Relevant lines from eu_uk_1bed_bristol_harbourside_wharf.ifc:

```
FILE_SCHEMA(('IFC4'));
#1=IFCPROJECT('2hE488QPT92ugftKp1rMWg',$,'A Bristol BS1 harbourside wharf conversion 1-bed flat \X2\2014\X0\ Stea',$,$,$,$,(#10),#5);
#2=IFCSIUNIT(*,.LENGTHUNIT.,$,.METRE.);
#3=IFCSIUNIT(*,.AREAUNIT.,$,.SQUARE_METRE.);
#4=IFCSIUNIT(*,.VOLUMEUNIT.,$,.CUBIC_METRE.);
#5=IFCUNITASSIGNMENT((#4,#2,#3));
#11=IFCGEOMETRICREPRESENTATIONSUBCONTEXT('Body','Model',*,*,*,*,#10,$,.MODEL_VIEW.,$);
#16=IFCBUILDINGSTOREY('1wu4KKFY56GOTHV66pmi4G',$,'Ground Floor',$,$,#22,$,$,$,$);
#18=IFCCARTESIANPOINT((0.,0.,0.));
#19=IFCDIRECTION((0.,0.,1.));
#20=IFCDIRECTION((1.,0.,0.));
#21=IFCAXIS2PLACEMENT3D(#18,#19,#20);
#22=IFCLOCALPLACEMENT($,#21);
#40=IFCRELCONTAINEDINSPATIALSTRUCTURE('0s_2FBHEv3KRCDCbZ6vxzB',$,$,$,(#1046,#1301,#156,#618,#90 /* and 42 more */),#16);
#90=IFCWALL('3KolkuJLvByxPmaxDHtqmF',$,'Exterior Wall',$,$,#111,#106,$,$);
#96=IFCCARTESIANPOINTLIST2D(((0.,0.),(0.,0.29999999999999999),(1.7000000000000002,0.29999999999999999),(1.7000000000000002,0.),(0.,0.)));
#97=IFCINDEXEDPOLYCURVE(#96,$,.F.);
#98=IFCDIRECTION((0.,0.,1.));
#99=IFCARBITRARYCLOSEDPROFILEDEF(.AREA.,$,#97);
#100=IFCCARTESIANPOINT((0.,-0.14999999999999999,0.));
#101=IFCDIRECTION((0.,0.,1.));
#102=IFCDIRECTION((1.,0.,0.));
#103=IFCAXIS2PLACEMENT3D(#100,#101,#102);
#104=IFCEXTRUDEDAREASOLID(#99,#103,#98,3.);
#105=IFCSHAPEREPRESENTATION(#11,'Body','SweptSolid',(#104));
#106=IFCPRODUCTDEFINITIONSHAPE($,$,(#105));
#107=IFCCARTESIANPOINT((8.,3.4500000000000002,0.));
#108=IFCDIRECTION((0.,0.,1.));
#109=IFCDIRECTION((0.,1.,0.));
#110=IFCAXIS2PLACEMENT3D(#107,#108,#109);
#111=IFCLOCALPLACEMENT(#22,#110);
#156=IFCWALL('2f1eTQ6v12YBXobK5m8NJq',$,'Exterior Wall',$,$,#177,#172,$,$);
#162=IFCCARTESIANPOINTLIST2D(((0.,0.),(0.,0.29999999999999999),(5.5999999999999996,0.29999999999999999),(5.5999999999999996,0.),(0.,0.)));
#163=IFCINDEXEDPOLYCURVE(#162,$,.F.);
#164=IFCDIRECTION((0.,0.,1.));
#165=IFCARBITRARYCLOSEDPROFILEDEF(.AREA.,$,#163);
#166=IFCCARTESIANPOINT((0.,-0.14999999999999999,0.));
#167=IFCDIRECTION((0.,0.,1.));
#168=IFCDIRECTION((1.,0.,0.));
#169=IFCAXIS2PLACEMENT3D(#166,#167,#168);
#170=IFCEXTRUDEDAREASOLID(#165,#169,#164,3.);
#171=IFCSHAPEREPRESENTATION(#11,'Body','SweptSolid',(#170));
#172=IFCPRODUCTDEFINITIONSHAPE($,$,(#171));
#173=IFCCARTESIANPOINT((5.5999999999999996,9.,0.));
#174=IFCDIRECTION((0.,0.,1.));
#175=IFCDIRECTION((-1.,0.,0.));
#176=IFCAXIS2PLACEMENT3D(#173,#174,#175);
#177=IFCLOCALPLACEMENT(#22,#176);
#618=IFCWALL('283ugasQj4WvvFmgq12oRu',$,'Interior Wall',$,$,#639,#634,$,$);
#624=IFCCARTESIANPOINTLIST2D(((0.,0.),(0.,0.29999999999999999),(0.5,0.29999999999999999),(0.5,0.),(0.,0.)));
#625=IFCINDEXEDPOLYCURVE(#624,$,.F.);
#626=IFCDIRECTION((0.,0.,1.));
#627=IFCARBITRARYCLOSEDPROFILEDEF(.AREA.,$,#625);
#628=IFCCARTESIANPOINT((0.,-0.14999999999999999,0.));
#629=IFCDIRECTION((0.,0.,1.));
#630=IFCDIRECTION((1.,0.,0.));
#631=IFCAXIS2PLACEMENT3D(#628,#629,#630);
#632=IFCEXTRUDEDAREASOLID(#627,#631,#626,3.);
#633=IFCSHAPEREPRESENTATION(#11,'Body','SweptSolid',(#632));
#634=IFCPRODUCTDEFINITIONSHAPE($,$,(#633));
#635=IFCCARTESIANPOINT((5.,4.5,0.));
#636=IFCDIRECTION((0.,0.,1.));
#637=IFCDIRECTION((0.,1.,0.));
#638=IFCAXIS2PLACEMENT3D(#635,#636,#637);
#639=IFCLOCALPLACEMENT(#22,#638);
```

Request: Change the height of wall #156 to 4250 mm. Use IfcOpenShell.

```python
import ifcopenshell
import ifcopenshell.geom
import ifcopenshell.util.representation
import ifcopenshell.util.shape
import ifcopenshell.util.unit

model = ifcopenshell.open("eu_uk_1bed_bristol_harbourside_wharf.ifc")
unit_scale = ifcopenshell.util.unit.calculate_unit_scale(model)
settings = ifcopenshell.geom.settings()


def volume(element):
    """Net volume in cubic metres, openings subtracted."""
    shape = ifcopenshell.geom.create_shape(settings, element)
    return ifcopenshell.util.shape.get_volume(shape.geometry)


wall = model.by_id(156)
before = volume(wall)

body = ifcopenshell.util.representation.get_representation(wall, "Model", "Body")
solid = body.Items[0]
old_height = solid.Depth
solid.Depth = 4.25 / unit_scale
after = volume(wall)

print(f"height {old_height:g} -> {solid.Depth:g}, volume {before:.3f} -> {after:.3f} m3")

model.write("eu_uk_1bed_bristol_harbourside_wharf_updated.ifc")
```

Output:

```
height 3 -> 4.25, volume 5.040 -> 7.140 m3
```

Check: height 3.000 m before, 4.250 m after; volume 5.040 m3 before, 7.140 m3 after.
